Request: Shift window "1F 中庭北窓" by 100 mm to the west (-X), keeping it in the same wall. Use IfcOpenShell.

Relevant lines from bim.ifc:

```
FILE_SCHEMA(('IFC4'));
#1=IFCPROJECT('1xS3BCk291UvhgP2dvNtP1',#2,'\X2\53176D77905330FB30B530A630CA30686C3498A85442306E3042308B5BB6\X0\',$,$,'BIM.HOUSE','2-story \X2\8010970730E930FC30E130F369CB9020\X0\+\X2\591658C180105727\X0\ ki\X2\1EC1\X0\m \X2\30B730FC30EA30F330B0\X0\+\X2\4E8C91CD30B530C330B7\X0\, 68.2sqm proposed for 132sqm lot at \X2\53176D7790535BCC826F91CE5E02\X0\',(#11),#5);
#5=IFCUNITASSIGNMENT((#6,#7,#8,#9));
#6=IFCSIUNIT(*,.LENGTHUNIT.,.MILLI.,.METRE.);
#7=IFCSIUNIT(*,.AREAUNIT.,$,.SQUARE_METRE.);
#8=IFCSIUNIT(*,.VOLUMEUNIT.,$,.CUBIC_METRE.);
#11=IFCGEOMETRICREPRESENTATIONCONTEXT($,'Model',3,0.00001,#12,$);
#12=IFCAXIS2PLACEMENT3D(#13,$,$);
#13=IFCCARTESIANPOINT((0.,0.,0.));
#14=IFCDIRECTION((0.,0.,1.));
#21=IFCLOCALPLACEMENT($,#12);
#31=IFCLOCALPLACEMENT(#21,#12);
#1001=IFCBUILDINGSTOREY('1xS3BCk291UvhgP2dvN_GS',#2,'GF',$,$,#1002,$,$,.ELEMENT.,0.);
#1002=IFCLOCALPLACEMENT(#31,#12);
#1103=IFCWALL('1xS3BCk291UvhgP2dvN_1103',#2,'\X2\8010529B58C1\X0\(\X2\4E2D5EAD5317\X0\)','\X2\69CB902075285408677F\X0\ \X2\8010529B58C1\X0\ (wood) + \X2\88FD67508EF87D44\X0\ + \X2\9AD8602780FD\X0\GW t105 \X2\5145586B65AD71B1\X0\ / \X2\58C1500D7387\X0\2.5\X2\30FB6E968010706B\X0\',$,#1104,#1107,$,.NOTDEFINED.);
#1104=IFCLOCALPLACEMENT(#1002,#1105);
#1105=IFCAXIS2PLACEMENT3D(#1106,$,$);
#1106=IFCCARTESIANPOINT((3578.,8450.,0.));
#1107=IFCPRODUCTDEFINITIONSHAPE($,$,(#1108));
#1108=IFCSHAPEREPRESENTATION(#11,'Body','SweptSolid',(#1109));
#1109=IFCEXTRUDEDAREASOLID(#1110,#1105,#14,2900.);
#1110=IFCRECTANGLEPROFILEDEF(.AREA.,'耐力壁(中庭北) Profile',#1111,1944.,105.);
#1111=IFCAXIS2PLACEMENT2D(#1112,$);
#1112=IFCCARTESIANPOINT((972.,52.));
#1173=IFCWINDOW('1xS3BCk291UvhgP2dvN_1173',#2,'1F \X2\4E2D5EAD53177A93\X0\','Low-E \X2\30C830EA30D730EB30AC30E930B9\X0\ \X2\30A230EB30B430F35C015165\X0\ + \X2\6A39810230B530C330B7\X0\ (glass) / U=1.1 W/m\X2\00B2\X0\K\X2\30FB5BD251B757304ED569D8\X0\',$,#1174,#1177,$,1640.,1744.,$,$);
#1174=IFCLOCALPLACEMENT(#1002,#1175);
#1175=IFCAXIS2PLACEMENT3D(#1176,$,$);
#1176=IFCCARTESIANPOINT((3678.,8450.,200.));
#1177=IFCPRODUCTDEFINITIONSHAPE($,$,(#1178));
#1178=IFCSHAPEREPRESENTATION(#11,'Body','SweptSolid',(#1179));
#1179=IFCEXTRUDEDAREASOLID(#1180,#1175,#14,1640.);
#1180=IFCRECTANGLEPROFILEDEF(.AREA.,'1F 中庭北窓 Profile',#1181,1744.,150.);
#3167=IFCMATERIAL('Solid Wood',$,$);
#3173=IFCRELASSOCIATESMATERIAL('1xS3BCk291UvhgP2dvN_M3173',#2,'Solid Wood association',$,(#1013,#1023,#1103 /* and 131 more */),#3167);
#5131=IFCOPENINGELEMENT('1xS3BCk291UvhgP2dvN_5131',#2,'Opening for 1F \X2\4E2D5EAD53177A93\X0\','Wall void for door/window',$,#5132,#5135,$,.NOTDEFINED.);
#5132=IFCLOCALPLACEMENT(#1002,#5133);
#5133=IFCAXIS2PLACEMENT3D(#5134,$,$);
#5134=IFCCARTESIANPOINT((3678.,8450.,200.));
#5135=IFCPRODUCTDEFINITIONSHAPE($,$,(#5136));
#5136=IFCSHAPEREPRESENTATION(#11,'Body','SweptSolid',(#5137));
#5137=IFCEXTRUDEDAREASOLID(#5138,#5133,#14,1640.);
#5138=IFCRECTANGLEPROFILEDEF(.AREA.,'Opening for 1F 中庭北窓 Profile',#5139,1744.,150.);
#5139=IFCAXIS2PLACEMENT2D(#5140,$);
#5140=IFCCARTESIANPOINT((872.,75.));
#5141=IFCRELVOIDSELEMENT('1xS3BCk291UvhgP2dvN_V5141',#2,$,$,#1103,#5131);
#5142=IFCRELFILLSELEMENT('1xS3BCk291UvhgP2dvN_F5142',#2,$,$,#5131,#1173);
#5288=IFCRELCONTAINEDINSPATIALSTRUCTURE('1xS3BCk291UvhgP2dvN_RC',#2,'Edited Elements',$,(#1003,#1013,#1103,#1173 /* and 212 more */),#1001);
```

```python
import ifcopenshell
import ifcopenshell.api.geometry
import ifcopenshell.util.placement
import ifcopenshell.util.unit

model = ifcopenshell.open("bim.ifc")
unit_scale = ifcopenshell.util.unit.calculate_unit_scale(model)

window = model.by_id(1173)
opening = window.FillsVoids[0].RelatingOpeningElement
wall = opening.VoidsElements[0].RelatingBuildingElement

wall_matrix = ifcopenshell.util.placement.get_local_placement(wall.ObjectPlacement)
shift = wall_matrix[:3, 0] * -0.1 / unit_scale
before = ifcopenshell.util.placement.get_local_placement(window.ObjectPlacement)[:3, 3].copy()

# The window is not placed relative to its opening, so move both.
for product in (opening, window):
    matrix = ifcopenshell.util.placement.get_local_placement(product.ObjectPlacement)
    matrix[:3, 3] += shift
    ifcopenshell.api.geometry.edit_object_placement(model, product=product, matrix=matrix, is_si=False)

after = ifcopenshell.util.placement.get_local_placement(window.ObjectPlacement)[:3, 3]
print("window moved by", (after - before).round(3) + 0.0)

model.write("bim_v2.ifc")
```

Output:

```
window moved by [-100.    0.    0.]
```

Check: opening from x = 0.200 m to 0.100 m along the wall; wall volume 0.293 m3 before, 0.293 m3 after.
